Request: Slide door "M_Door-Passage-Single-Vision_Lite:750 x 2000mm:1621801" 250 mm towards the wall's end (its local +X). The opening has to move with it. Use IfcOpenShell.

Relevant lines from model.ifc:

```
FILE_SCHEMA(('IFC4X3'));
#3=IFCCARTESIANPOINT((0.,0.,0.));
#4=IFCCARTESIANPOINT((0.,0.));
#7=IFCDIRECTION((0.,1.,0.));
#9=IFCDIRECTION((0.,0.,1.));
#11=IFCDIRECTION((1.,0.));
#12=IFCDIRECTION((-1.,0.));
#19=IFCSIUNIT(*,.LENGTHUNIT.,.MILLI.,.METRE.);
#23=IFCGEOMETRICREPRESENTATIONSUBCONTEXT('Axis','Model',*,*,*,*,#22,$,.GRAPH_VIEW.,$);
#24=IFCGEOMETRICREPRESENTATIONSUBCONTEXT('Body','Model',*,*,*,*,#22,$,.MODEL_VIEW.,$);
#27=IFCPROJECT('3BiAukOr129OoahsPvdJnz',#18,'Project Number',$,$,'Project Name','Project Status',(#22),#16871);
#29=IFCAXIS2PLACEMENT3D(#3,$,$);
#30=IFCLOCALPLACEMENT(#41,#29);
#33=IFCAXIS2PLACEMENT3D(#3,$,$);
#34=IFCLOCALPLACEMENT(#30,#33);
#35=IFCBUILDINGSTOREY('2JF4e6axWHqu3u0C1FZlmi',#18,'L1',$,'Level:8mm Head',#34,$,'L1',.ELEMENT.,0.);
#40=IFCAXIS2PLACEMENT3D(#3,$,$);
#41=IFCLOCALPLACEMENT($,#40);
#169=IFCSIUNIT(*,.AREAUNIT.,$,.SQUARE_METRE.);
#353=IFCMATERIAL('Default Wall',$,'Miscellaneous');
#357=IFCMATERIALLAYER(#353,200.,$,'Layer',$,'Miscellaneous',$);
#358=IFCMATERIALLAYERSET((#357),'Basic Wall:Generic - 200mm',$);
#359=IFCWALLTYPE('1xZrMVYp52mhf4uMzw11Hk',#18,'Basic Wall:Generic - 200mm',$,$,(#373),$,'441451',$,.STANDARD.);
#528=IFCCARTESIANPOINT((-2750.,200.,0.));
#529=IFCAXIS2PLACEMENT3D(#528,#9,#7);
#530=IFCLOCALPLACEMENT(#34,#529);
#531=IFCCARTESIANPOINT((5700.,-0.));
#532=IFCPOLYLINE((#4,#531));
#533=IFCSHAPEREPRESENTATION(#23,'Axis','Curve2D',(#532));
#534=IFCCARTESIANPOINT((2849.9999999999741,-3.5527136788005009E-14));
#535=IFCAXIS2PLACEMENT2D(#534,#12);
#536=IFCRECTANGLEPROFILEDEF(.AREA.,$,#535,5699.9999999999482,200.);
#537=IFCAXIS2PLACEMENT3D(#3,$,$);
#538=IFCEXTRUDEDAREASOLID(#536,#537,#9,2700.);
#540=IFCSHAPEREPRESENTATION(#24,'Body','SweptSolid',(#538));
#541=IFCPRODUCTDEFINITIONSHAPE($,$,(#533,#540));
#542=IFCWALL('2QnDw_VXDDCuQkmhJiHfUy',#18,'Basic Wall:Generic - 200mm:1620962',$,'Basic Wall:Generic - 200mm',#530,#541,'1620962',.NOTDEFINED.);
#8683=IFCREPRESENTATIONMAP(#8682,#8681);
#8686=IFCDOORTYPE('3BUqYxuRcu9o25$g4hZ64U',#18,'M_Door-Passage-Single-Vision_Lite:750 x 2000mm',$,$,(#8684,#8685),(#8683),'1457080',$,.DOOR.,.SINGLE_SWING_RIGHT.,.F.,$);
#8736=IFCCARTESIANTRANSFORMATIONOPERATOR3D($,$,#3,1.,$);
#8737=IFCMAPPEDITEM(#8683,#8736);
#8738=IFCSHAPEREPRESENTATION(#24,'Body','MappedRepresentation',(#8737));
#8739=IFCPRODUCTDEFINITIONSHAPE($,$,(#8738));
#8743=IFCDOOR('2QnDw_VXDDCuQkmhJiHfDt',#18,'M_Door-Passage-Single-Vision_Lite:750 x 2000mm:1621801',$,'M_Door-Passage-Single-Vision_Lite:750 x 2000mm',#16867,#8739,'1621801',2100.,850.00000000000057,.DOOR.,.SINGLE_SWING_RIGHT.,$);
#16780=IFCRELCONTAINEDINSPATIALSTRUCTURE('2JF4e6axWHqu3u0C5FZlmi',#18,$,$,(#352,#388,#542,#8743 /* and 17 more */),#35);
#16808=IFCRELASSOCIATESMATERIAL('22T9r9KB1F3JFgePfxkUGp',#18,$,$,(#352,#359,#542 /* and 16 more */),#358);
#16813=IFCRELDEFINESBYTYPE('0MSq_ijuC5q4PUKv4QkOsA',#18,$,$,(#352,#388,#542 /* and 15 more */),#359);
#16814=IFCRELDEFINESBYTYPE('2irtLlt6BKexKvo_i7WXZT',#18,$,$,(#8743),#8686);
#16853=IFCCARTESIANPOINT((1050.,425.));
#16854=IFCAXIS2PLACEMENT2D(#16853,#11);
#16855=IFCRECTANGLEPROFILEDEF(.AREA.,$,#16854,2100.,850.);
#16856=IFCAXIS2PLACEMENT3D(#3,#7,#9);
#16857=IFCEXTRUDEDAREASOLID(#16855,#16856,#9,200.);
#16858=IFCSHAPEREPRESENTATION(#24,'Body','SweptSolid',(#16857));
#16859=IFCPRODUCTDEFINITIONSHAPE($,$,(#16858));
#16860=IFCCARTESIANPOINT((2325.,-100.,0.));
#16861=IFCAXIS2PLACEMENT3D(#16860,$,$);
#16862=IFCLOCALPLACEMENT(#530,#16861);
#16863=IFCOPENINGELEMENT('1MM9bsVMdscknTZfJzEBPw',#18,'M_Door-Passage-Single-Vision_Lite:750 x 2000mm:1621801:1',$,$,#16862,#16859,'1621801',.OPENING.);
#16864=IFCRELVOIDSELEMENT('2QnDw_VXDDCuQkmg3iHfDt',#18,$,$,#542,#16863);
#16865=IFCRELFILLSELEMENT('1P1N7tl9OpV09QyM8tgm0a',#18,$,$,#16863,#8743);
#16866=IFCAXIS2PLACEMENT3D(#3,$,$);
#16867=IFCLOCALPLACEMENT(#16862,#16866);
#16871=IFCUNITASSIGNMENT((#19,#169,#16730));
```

```python
import ifcopenshell
import ifcopenshell.api.geometry
import ifcopenshell.util.placement

model = ifcopenshell.open("model.ifc")

door = model.by_id(8743)
opening = door.FillsVoids[0].RelatingOpeningElement
wall = opening.VoidsElements[0].RelatingBuildingElement

wall_matrix = ifcopenshell.util.placement.get_local_placement(wall.ObjectPlacement)
shift = wall_matrix[:3, 0] * 250.0
before = ifcopenshell.util.placement.get_local_placement(door.ObjectPlacement)[:3, 3].copy()

# The door is placed relative to its opening, so it follows when the opening moves.
matrix = ifcopenshell.util.placement.get_local_placement(opening.ObjectPlacement)
matrix[:3, 3] += shift
ifcopenshell.api.geometry.edit_object_placement(
    model, product=opening, matrix=matrix, is_si=False, should_transform_children=True
)

after = ifcopenshell.util.placement.get_local_placement(door.ObjectPlacement)[:3, 3]
print("door moved by", (after - before).round(3) + 0.0)

model.write("model_v2.ifc")
```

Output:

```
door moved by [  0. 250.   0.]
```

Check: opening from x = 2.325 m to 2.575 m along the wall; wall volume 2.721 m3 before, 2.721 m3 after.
